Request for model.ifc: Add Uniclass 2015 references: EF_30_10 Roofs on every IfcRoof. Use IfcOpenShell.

First a look at what the model holds.

```python
import ifcopenshell

model = ifcopenshell.open("model.ifc")
print(model.schema)
print("classifications:", [c.Name for c in model.by_type("IfcClassification")])
for ifc_class in ("IfcDoor", "IfcRoof", "IfcStair", "IfcWall", "IfcWindow"):
    print(ifc_class, len(model.by_type(ifc_class)))
```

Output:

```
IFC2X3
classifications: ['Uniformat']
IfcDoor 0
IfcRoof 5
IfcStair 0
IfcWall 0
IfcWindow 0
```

```python
import ifcopenshell
import ifcopenshell.api.classification

model = ifcopenshell.open("model.ifc")

# IFC2X3 requires Source and Edition and has no link from the project to the system.
system = model.create_entity("IfcClassification", Source="NBS", Edition="2015", Name="Uniclass 2015")

codes = {
    "IfcRoof": ("EF_30_10", "Roofs"),
}
for ifc_class, (code, name) in codes.items():
    products = model.by_type(ifc_class)
    ifcopenshell.api.classification.add_reference(
        model, products=products, classification=system, identification=code, name=name
    )
    print(code, len(products))

model.write("model_v2.ifc")
```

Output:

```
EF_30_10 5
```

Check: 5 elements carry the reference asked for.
